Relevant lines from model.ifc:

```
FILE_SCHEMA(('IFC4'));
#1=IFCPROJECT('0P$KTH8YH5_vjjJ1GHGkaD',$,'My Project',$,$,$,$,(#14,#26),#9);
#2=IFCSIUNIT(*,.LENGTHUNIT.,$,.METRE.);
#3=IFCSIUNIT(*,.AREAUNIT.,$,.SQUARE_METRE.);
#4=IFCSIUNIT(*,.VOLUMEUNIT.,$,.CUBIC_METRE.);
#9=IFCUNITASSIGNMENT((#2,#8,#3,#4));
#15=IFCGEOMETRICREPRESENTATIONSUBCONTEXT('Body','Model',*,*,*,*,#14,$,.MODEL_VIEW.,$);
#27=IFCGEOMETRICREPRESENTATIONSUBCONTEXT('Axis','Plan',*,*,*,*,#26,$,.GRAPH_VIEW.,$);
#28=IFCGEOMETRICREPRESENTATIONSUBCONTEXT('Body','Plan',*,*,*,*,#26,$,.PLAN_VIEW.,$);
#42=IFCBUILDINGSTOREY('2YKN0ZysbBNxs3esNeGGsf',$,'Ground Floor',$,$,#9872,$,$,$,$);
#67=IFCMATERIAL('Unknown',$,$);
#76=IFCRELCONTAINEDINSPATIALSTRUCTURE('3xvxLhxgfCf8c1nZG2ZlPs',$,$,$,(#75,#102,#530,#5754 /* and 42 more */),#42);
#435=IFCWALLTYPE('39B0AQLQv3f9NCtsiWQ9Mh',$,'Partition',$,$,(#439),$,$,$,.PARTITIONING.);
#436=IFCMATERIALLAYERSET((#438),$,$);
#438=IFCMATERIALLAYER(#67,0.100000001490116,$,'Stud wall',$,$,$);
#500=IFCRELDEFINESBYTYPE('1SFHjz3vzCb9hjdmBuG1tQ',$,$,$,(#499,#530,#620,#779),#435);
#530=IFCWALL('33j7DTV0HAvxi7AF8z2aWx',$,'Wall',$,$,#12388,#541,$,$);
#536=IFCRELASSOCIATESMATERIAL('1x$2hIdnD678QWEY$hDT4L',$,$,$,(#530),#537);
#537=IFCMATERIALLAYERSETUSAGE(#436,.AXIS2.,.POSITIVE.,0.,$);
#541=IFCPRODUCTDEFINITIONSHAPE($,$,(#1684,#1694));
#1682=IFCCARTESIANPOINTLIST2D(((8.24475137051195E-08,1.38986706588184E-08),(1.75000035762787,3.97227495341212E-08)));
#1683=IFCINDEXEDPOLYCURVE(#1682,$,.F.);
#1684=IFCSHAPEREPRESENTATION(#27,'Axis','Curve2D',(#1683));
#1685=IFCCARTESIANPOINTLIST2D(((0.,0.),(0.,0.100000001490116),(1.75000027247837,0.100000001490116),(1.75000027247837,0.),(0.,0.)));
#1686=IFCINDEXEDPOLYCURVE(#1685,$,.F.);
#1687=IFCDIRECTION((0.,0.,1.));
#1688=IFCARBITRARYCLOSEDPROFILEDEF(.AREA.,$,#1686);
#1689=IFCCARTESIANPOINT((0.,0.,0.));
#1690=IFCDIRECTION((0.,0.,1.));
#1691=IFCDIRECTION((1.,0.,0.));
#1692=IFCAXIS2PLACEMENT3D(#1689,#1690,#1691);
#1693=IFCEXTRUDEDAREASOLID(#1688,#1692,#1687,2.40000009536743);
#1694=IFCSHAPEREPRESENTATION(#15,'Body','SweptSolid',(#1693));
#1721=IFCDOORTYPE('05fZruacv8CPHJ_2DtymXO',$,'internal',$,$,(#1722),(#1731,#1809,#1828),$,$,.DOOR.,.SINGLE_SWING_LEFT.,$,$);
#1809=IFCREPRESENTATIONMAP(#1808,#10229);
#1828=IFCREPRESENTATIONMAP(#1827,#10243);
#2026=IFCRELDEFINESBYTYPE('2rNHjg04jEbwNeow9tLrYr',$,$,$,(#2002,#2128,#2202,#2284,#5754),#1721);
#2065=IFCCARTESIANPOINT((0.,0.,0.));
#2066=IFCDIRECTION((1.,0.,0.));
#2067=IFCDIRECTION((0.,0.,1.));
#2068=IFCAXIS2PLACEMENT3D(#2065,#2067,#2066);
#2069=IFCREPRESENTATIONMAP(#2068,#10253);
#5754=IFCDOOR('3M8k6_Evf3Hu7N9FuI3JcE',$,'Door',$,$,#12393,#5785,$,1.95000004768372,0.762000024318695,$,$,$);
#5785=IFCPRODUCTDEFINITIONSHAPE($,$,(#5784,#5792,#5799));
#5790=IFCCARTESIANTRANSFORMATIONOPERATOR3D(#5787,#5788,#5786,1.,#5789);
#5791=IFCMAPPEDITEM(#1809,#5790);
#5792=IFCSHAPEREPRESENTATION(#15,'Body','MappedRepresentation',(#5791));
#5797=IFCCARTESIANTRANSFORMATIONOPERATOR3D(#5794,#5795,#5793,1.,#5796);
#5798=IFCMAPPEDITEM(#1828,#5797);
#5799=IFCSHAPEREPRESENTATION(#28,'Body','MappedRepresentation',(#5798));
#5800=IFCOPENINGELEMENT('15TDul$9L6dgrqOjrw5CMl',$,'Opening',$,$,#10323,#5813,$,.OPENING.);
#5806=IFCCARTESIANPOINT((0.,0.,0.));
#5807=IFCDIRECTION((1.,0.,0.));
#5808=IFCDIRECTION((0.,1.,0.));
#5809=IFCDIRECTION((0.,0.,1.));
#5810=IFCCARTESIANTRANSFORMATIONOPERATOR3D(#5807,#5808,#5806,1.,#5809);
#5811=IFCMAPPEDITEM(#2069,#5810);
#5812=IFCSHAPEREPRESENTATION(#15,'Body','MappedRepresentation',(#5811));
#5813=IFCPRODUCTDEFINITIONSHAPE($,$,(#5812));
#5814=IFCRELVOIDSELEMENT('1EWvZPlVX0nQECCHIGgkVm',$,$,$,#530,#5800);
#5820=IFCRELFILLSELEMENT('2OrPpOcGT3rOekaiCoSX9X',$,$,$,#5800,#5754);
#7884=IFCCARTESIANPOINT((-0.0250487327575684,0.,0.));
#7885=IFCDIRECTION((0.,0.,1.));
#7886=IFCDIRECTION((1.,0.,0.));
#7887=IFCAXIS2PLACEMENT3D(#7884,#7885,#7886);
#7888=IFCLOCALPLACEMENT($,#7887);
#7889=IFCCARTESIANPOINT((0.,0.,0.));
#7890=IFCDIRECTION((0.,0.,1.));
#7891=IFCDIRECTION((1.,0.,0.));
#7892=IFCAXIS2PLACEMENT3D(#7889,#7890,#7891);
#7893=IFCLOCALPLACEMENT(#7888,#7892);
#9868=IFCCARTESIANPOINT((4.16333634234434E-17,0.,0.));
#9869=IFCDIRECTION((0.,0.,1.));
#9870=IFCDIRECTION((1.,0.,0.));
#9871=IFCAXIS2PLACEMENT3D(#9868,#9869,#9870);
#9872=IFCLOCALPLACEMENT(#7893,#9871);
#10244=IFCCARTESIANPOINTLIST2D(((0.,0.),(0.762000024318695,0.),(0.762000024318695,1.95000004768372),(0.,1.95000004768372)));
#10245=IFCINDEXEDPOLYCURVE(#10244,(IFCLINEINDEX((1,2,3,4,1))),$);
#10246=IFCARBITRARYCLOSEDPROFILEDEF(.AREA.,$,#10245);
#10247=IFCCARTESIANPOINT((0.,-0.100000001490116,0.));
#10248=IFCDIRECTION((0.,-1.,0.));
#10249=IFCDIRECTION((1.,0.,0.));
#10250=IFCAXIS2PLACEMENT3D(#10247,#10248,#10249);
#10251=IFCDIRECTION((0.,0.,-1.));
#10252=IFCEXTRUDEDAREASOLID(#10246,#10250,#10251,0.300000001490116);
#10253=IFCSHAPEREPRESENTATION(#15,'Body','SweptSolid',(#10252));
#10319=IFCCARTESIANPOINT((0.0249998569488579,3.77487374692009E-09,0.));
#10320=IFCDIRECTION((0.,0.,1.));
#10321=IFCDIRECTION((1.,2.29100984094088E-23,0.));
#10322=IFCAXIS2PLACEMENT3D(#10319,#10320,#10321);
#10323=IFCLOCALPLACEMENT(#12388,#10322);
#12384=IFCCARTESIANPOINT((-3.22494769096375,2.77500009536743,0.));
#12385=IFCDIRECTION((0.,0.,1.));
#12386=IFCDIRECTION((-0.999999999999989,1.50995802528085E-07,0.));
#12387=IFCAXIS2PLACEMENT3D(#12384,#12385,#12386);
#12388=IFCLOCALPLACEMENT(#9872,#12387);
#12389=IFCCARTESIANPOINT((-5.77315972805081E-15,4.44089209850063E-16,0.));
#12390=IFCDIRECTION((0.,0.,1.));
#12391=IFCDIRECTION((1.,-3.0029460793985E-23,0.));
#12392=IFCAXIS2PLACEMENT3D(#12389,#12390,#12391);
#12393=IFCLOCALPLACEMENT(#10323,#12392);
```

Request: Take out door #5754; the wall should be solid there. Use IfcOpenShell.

```python
import ifcopenshell
import ifcopenshell.api.feature
import ifcopenshell.api.root
import ifcopenshell.geom
import ifcopenshell.util.shape

model = ifcopenshell.open("model.ifc")
settings = ifcopenshell.geom.settings()


def volume(element):
    """Net volume in cubic metres, openings subtracted."""
    shape = ifcopenshell.geom.create_shape(settings, element)
    return ifcopenshell.util.shape.get_volume(shape.geometry)


door = model.by_guid("3M8k6_Evf3Hu7N9FuI3JcE")
opening = door.FillsVoids[0].RelatingOpeningElement
wall = opening.VoidsElements[0].RelatingBuildingElement
before = volume(wall)

ifcopenshell.api.root.remove_product(model, product=door)
ifcopenshell.api.feature.remove_feature(model, feature=opening)

after = volume(wall)

print(f"wall volume {before:.3f} -> {after:.3f} m3")

model.write("model_updated.ifc")
```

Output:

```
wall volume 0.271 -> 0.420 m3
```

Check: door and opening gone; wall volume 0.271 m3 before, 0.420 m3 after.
